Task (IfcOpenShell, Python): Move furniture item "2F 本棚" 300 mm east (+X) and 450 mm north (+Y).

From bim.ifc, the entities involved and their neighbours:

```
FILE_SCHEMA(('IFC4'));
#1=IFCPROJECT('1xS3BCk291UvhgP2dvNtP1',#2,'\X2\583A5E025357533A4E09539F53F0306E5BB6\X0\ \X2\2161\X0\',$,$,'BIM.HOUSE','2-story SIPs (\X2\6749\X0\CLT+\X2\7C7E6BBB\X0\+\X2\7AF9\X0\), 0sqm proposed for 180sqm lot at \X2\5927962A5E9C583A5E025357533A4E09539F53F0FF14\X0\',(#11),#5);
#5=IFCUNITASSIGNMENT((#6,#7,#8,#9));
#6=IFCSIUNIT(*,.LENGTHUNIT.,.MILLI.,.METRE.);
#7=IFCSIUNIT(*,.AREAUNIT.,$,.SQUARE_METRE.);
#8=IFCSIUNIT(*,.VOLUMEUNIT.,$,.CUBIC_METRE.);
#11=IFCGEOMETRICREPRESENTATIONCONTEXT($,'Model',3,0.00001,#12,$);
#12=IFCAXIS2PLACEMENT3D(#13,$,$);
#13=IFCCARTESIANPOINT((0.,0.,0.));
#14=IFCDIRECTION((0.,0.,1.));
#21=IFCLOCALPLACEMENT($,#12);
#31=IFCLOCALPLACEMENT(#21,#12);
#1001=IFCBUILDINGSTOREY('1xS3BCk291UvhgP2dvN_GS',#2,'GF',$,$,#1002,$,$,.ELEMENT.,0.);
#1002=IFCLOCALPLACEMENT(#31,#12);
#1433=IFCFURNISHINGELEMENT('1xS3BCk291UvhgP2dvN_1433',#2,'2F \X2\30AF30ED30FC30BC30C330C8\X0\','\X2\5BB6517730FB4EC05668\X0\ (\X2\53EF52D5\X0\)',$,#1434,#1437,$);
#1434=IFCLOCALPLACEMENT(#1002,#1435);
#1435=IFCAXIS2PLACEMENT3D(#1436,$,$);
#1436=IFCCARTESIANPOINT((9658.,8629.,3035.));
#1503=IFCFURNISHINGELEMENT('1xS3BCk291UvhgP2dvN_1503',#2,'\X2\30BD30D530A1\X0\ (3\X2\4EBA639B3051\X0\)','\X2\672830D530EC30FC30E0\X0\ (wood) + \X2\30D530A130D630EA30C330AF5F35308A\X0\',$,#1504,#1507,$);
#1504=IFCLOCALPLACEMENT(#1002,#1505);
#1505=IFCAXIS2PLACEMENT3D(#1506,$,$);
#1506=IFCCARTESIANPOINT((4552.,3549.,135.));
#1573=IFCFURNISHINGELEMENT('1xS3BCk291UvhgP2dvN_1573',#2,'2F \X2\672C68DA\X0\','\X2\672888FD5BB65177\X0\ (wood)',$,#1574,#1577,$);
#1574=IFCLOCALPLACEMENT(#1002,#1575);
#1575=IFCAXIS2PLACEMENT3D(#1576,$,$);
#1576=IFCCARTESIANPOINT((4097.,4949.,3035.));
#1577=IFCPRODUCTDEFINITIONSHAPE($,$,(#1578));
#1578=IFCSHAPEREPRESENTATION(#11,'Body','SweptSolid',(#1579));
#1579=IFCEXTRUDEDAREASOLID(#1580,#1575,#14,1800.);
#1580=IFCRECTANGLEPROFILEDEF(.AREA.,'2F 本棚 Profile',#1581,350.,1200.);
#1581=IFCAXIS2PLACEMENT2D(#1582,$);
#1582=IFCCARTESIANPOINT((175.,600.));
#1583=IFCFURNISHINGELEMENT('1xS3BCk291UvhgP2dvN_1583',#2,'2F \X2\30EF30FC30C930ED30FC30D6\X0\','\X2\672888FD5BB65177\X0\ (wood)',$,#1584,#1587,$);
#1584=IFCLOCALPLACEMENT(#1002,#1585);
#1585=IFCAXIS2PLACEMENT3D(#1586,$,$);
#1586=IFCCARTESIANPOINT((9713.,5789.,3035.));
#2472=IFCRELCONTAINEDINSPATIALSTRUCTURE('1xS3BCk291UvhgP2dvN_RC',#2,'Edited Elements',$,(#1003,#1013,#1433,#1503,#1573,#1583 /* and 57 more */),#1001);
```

```python
import ifcopenshell
import ifcopenshell.api.geometry
import ifcopenshell.util.placement

model = ifcopenshell.open("bim.ifc")

item = model.by_guid("1xS3BCk291UvhgP2dvN_1573")
matrix = ifcopenshell.util.placement.get_local_placement(item.ObjectPlacement)
matrix[0, 3] += 300.0
matrix[1, 3] += 450.0
ifcopenshell.api.geometry.edit_object_placement(model, product=item, matrix=matrix, is_si=False)

print(ifcopenshell.util.placement.get_local_placement(item.ObjectPlacement).round(3) + 0.0)

model.write("bim_updated.ifc")
```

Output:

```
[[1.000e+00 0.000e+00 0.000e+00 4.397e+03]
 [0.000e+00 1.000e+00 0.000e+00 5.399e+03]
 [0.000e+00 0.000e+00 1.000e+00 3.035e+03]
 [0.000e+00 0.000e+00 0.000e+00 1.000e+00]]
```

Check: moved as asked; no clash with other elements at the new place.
